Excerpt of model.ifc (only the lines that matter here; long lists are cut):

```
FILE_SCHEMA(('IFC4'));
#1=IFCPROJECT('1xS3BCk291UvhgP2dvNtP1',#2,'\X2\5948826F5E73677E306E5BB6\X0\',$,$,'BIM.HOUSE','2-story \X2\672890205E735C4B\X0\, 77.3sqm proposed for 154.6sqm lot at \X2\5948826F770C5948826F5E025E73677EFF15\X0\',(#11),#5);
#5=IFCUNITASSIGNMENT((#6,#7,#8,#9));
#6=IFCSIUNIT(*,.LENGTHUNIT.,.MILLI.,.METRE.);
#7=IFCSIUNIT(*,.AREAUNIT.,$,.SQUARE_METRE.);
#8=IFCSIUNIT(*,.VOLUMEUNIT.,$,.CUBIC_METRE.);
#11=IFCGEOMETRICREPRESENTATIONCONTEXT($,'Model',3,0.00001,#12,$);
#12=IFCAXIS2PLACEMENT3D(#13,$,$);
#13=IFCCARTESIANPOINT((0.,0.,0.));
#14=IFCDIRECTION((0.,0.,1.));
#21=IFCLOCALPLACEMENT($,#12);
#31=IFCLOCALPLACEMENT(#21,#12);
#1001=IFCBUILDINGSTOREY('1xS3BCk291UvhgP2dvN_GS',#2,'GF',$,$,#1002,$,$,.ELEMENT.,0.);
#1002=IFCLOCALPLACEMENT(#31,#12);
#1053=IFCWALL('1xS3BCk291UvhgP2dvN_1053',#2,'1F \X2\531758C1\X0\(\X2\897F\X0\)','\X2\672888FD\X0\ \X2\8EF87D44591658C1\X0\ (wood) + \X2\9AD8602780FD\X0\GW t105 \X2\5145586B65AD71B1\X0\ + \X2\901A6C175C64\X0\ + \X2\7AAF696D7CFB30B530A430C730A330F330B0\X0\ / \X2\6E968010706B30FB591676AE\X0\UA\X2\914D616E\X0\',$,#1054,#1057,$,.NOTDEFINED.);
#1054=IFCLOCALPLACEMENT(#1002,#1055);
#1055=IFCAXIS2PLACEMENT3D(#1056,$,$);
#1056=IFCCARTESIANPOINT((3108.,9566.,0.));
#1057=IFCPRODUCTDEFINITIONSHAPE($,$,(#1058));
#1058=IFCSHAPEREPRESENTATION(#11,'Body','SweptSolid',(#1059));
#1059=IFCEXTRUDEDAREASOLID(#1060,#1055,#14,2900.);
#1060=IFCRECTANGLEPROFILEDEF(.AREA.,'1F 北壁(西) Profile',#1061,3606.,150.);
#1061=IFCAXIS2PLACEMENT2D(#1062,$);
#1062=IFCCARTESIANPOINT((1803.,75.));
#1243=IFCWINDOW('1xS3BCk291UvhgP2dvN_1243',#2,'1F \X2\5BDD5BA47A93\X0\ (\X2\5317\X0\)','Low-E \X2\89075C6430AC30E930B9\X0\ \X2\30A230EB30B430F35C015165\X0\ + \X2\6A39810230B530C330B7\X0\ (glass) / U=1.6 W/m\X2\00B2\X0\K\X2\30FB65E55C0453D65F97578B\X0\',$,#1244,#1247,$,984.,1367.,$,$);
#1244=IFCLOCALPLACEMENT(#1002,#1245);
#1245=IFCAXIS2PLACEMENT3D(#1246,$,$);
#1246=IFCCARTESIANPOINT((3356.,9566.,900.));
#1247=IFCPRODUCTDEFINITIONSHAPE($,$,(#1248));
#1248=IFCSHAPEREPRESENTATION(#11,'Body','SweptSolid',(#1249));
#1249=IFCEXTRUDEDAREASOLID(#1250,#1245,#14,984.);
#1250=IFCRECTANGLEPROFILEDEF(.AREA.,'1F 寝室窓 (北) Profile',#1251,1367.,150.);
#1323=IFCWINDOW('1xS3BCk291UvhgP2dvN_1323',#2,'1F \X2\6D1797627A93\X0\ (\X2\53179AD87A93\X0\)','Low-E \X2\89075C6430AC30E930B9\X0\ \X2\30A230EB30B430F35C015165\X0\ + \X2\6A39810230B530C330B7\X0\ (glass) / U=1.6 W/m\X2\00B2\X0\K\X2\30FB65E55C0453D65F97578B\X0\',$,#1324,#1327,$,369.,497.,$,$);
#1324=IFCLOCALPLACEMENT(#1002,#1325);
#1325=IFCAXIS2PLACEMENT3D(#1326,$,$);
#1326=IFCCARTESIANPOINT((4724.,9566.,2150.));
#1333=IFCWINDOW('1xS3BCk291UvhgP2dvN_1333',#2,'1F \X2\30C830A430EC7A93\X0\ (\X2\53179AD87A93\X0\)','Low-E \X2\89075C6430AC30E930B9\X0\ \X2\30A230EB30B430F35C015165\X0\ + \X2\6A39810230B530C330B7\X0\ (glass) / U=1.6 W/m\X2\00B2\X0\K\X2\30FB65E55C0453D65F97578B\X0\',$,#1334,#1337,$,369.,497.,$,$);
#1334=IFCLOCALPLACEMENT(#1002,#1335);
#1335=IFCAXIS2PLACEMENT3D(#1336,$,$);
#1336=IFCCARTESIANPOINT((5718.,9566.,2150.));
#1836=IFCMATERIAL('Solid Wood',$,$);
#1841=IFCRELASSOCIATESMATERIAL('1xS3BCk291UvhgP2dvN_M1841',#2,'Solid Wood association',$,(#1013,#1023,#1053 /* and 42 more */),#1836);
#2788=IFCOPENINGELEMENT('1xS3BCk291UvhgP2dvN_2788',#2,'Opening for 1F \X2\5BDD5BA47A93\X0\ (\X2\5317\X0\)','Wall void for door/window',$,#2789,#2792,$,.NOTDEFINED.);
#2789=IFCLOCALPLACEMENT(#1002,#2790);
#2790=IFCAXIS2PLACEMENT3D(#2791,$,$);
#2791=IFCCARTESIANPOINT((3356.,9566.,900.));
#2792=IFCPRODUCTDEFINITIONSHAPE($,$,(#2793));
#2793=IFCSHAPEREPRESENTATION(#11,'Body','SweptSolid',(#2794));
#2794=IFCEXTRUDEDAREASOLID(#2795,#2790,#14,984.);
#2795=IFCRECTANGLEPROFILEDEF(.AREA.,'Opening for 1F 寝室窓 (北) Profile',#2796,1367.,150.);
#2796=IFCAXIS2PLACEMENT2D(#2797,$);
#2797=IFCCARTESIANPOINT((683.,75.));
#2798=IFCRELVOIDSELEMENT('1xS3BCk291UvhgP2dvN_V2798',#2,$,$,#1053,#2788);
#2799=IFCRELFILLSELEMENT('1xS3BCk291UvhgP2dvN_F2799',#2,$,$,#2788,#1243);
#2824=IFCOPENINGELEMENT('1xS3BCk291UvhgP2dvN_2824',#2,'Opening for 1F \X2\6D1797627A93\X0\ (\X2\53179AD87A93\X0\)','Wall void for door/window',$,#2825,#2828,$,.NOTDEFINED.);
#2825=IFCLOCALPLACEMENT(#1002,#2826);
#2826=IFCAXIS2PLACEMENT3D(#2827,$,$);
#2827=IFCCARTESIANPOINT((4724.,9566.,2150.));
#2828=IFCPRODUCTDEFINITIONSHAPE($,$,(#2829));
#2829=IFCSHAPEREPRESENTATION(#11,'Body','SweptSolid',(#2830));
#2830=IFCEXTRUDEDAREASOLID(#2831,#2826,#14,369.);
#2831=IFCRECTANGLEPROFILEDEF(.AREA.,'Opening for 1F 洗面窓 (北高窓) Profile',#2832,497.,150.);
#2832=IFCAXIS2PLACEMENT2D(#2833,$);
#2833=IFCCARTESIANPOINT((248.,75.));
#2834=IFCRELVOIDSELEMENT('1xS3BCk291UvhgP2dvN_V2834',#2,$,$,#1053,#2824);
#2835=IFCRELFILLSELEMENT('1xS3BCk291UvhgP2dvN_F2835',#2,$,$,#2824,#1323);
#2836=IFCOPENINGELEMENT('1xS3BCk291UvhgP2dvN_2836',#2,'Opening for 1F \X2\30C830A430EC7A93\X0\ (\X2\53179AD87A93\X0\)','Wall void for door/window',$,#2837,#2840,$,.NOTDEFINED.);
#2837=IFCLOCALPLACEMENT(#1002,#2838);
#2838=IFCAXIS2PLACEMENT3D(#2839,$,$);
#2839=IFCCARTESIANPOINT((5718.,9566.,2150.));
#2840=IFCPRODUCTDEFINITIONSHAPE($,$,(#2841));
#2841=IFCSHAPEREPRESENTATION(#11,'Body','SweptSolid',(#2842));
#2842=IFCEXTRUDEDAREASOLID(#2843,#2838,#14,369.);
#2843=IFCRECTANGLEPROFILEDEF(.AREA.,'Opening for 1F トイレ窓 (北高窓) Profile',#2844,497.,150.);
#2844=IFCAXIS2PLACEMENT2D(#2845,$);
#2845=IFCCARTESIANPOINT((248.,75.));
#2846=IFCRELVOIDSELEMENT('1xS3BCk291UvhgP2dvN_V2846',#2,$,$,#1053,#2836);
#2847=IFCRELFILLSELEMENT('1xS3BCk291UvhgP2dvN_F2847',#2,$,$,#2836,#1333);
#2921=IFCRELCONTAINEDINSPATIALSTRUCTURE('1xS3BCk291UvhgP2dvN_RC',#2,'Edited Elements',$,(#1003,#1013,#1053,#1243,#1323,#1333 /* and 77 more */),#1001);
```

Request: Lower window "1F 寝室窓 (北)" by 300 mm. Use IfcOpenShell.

```python
import numpy as np
import ifcopenshell
import ifcopenshell.api.geometry
import ifcopenshell.util.placement
import ifcopenshell.util.unit

model = ifcopenshell.open("model.ifc")
unit_scale = ifcopenshell.util.unit.calculate_unit_scale(model)

window = model.by_id(1243)
opening = window.FillsVoids[0].RelatingOpeningElement
dz = -300.0

shift = np.array([0.0, 0.0, dz])
# The window is not placed relative to its opening, so move both.
for product in (opening, window):
    matrix = ifcopenshell.util.placement.get_local_placement(product.ObjectPlacement)
    matrix[:3, 3] += shift
    ifcopenshell.api.geometry.edit_object_placement(model, product=product, matrix=matrix, is_si=False)

print(f"moved by {dz * unit_scale:+.3f} m")

model.write("model_rev.ifc")
```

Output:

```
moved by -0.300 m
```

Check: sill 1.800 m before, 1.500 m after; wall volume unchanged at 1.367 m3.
